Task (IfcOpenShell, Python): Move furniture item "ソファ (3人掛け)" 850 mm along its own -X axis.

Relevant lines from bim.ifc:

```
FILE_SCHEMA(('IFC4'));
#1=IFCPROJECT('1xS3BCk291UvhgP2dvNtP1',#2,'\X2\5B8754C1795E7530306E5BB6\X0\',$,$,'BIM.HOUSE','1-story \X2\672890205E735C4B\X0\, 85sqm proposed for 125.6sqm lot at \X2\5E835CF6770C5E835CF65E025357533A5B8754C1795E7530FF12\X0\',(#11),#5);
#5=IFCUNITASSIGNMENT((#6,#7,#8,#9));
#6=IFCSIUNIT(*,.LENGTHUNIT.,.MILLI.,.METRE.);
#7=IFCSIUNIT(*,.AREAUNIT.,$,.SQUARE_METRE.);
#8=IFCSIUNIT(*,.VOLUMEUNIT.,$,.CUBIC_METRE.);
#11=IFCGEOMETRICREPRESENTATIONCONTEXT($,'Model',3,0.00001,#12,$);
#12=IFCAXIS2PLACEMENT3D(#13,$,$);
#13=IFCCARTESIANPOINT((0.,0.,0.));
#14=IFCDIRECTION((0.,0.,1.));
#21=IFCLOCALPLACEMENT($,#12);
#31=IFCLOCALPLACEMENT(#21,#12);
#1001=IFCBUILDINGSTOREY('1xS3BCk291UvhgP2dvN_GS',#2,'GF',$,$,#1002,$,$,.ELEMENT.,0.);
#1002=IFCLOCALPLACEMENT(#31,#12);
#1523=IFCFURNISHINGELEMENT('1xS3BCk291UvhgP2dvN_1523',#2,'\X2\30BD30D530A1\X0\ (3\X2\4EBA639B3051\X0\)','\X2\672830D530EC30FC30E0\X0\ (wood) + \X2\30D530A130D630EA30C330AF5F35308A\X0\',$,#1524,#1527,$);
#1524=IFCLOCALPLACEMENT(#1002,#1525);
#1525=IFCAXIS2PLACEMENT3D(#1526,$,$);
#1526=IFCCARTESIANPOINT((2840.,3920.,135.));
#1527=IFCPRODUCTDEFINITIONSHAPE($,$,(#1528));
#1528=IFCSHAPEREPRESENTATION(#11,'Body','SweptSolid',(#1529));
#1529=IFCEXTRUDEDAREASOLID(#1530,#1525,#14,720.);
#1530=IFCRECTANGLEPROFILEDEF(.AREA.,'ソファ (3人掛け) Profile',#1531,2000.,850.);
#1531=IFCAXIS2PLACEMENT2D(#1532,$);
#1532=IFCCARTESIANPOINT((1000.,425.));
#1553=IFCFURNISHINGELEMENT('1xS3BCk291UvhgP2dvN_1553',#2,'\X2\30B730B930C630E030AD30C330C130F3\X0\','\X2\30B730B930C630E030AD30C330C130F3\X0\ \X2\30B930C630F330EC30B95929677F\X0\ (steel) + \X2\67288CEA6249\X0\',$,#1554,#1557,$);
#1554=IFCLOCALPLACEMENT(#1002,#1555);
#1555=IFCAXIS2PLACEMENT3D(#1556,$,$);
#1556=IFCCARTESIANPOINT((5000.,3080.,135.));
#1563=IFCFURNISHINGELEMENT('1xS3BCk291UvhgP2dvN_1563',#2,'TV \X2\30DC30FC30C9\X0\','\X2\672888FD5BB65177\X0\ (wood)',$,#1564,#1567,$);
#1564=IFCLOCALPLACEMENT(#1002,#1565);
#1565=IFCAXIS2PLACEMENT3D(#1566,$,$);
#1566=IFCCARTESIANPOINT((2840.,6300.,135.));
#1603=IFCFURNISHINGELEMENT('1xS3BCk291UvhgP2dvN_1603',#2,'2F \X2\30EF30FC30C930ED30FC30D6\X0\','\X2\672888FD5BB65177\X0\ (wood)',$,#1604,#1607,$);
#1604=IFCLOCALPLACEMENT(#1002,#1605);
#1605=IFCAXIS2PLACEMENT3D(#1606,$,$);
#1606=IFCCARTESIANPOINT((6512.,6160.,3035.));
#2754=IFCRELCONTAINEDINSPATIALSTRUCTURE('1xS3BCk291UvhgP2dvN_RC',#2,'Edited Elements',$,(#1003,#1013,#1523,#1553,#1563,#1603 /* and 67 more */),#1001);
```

```python
import ifcopenshell
import ifcopenshell.api.geometry
import ifcopenshell.util.placement
import ifcopenshell.util.unit

model = ifcopenshell.open("bim.ifc")
unit_scale = ifcopenshell.util.unit.calculate_unit_scale(model)

item = model.by_id(1523)
matrix = ifcopenshell.util.placement.get_local_placement(item.ObjectPlacement)
matrix[:3, 3] -= matrix[:3, 0] * 0.85 / unit_scale
ifcopenshell.api.geometry.edit_object_placement(model, product=item, matrix=matrix, is_si=False)

print(ifcopenshell.util.placement.get_local_placement(item.ObjectPlacement).round(3) + 0.0)

model.write("bim_edited.ifc")
```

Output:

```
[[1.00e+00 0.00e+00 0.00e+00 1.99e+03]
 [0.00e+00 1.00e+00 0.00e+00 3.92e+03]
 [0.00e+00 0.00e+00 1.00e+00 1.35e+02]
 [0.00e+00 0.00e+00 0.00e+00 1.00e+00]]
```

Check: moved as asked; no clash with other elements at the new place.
